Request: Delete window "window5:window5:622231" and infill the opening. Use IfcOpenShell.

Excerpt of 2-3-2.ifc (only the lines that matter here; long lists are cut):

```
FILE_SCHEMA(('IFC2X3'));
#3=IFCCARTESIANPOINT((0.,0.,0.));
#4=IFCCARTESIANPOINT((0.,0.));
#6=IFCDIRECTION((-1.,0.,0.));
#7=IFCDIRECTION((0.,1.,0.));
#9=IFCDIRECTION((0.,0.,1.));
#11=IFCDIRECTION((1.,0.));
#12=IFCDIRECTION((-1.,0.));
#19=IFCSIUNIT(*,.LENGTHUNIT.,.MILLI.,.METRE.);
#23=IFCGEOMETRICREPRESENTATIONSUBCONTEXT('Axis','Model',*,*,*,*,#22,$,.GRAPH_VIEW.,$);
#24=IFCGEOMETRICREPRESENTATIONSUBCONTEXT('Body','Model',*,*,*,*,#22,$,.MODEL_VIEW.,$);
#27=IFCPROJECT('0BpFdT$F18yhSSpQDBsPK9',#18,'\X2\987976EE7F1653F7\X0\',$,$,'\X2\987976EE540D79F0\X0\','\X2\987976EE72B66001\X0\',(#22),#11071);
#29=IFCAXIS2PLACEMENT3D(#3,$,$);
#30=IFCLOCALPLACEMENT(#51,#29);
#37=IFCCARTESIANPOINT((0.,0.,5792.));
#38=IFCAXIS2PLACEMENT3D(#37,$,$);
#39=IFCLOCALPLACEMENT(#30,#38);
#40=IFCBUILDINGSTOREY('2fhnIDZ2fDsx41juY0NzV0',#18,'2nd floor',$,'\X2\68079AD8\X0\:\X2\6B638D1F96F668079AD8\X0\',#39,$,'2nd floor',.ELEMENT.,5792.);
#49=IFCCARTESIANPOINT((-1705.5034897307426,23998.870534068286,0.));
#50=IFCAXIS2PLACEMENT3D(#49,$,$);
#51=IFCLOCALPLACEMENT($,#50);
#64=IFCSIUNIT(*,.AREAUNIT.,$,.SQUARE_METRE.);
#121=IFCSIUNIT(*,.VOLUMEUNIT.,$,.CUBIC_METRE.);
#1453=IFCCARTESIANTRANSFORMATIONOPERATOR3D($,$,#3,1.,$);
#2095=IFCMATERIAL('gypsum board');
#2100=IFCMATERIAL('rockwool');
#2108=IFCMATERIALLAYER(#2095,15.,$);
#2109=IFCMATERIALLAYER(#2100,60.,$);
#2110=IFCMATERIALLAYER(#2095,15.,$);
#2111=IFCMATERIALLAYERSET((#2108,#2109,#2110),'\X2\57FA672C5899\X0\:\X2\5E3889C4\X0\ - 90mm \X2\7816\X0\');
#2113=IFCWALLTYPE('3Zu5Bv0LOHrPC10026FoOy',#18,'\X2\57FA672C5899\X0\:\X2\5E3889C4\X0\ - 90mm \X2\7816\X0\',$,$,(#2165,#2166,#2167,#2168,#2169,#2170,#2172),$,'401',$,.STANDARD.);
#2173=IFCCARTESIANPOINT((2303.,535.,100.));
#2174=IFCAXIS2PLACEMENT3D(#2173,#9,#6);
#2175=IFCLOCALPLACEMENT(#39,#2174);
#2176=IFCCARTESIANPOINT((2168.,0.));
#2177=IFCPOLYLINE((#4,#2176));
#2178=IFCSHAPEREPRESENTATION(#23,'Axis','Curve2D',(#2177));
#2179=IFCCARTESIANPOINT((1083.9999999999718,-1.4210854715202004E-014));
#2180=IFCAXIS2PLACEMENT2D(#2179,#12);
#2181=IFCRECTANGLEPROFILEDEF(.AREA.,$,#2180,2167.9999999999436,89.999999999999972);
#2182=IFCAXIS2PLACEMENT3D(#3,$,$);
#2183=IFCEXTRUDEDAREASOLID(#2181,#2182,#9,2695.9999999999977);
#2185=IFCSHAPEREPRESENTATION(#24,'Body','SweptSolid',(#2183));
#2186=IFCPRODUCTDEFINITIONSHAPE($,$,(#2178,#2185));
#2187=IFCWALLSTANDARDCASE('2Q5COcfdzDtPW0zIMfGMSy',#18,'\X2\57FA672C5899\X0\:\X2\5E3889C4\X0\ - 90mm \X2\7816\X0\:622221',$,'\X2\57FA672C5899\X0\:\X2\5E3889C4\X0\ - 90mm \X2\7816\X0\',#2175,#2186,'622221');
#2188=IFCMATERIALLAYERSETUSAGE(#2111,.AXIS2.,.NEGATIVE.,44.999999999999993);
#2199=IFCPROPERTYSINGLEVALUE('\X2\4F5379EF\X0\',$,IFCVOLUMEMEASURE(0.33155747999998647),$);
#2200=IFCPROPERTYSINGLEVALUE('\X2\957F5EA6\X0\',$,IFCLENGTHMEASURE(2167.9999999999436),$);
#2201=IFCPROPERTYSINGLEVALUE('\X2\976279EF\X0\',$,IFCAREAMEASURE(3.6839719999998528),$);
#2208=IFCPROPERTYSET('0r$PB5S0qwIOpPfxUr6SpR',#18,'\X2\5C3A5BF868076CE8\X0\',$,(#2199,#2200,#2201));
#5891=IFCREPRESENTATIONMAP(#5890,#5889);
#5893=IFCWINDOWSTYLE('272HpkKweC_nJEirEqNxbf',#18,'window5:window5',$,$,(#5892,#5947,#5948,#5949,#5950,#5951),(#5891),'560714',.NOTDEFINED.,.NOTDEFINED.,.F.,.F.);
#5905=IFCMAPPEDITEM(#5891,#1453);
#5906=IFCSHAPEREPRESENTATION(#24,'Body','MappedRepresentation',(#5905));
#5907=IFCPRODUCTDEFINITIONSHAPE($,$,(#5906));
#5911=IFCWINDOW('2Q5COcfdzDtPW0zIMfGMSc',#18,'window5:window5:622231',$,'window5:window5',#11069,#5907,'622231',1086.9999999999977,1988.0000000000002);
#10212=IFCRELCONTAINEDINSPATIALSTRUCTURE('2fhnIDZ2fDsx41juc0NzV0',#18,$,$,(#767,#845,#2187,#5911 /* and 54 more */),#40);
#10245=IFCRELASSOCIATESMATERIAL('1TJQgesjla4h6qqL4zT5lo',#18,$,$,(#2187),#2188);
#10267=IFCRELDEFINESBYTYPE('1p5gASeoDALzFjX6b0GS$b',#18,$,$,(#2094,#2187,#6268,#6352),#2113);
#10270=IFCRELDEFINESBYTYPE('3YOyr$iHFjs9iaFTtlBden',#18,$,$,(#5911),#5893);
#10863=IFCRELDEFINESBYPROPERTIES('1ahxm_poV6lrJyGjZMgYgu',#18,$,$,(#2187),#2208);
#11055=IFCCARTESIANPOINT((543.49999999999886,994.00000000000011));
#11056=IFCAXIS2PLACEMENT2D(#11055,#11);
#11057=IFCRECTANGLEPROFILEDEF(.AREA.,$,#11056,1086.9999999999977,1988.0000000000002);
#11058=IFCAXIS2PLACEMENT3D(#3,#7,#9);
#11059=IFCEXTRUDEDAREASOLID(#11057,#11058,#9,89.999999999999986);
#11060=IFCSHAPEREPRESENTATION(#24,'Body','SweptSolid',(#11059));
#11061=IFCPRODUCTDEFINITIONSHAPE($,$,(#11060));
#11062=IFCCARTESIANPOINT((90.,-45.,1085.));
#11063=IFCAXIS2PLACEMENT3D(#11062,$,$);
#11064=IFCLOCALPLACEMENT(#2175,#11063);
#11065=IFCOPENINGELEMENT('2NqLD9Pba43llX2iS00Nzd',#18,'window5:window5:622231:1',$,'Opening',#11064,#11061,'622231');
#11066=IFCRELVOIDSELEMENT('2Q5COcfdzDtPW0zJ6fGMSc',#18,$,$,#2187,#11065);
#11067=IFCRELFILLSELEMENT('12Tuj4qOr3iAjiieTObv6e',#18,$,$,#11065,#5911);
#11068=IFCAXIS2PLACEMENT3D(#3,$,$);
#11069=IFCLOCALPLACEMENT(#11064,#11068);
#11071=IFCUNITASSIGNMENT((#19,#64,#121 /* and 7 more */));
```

```python
import ifcopenshell
import ifcopenshell.api.feature
import ifcopenshell.api.pset
import ifcopenshell.api.root
import ifcopenshell.geom
import ifcopenshell.util.element
import ifcopenshell.util.shape
import ifcopenshell.util.unit

model = ifcopenshell.open("2-3-2.ifc")
area_scale = ifcopenshell.util.unit.calculate_unit_scale(model, "AREAUNIT")
volume_scale = ifcopenshell.util.unit.calculate_unit_scale(model, "VOLUMEUNIT")
settings = ifcopenshell.geom.settings()


def volume(element):
    """Net volume in cubic metres, openings subtracted."""
    shape = ifcopenshell.geom.create_shape(settings, element)
    return ifcopenshell.util.shape.get_volume(shape.geometry)


window = model.by_guid("2Q5COcfdzDtPW0zIMfGMSc")
opening = window.FillsVoids[0].RelatingOpeningElement
wall = opening.VoidsElements[0].RelatingBuildingElement
before = volume(wall)

ifcopenshell.api.root.remove_product(model, product=window)
ifcopenshell.api.feature.remove_feature(model, feature=opening)

after = volume(wall)
thickness = 0.09  # wall thickness in metres

# Update the wall's stored quantities.
pset = model.by_id(ifcopenshell.util.element.get_pset(wall, "尺寸标注", should_inherit=False)["id"])
ifcopenshell.api.pset.edit_pset(model, pset=pset, properties={
    "体积": model.create_entity("IfcVolumeMeasure", after / volume_scale),
    "面积": model.create_entity("IfcAreaMeasure", after / thickness / area_scale),
})

print(f"wall volume {before:.3f} -> {after:.3f} m3")

model.write("2-3-2_updated.ifc")
```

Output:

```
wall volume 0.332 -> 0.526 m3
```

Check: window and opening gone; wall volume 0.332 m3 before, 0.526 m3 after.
